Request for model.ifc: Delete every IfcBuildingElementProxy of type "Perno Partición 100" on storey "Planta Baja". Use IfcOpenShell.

First a look at what the model holds.

```python
import ifcopenshell
import ifcopenshell.util.element

model = ifcopenshell.open("model.ifc")
print(model.schema)
storey = next(s for s in model.by_type("IfcBuildingStorey") if s.Name == "Planta Baja")
proxies = [e for e in ifcopenshell.util.element.get_decomposition(storey) if e.is_a("IfcBuildingElementProxy")]
seen = {}
for e in proxies:
    element_type = ifcopenshell.util.element.get_type(e)
    name = element_type.Name if element_type not in (None, e) else None
    seen[name] = seen.get(name, 0) + 1
for name, count in sorted(seen.items(), key=str):
    print(count, "x", name)
```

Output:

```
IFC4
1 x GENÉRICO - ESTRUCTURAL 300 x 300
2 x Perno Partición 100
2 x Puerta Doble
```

```python
import ifcopenshell
import ifcopenshell.api.root
import ifcopenshell.util.element

model = ifcopenshell.open("model.ifc")

storey = next(s for s in model.by_type("IfcBuildingStorey") if s.Name == "Planta Baja")
proxies = [e for e in ifcopenshell.util.element.get_decomposition(storey) if e.is_a("IfcBuildingElementProxy")]
targets = [e for e in proxies if (t := ifcopenshell.util.element.get_type(e)) not in (None, e) and t.Name == "Perno Partición 100"]

for e in targets:
    ifcopenshell.api.root.remove_product(model, product=e)
print(len(targets), "removed")

model.write("model_v2.ifc")
```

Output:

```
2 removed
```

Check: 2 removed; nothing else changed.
